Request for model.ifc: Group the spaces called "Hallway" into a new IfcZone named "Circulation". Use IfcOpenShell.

First a look at what the model holds.

```python
import ifcopenshell

model = ifcopenshell.open("model.ifc")
print(model.schema)
seen = {}
for space in model.by_type("IfcSpace"):
    seen[space.LongName] = seen.get(space.LongName, 0) + 1
for name, count in sorted(seen.items(), key=str):
    print(count, "x", name)
print("zones:", [z.Name for z in model.by_type("IfcZone")][:20])
```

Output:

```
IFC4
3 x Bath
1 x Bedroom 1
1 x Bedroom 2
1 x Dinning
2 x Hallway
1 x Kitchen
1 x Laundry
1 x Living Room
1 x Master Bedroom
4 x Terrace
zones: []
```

```python
import ifcopenshell
import ifcopenshell.api.group
import ifcopenshell.api.root

model = ifcopenshell.open("model.ifc")

names = {"Hallway"}
spaces = [s for s in model.by_type("IfcSpace") if s.LongName in names]

zone = ifcopenshell.api.root.create_entity(model, ifc_class="IfcZone", name="Circulation")
ifcopenshell.api.group.assign_group(model, products=spaces, group=zone)
print(len(spaces), "spaces in", zone.Name)

model.write("model-out.ifc")
```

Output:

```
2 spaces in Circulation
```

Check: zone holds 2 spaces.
